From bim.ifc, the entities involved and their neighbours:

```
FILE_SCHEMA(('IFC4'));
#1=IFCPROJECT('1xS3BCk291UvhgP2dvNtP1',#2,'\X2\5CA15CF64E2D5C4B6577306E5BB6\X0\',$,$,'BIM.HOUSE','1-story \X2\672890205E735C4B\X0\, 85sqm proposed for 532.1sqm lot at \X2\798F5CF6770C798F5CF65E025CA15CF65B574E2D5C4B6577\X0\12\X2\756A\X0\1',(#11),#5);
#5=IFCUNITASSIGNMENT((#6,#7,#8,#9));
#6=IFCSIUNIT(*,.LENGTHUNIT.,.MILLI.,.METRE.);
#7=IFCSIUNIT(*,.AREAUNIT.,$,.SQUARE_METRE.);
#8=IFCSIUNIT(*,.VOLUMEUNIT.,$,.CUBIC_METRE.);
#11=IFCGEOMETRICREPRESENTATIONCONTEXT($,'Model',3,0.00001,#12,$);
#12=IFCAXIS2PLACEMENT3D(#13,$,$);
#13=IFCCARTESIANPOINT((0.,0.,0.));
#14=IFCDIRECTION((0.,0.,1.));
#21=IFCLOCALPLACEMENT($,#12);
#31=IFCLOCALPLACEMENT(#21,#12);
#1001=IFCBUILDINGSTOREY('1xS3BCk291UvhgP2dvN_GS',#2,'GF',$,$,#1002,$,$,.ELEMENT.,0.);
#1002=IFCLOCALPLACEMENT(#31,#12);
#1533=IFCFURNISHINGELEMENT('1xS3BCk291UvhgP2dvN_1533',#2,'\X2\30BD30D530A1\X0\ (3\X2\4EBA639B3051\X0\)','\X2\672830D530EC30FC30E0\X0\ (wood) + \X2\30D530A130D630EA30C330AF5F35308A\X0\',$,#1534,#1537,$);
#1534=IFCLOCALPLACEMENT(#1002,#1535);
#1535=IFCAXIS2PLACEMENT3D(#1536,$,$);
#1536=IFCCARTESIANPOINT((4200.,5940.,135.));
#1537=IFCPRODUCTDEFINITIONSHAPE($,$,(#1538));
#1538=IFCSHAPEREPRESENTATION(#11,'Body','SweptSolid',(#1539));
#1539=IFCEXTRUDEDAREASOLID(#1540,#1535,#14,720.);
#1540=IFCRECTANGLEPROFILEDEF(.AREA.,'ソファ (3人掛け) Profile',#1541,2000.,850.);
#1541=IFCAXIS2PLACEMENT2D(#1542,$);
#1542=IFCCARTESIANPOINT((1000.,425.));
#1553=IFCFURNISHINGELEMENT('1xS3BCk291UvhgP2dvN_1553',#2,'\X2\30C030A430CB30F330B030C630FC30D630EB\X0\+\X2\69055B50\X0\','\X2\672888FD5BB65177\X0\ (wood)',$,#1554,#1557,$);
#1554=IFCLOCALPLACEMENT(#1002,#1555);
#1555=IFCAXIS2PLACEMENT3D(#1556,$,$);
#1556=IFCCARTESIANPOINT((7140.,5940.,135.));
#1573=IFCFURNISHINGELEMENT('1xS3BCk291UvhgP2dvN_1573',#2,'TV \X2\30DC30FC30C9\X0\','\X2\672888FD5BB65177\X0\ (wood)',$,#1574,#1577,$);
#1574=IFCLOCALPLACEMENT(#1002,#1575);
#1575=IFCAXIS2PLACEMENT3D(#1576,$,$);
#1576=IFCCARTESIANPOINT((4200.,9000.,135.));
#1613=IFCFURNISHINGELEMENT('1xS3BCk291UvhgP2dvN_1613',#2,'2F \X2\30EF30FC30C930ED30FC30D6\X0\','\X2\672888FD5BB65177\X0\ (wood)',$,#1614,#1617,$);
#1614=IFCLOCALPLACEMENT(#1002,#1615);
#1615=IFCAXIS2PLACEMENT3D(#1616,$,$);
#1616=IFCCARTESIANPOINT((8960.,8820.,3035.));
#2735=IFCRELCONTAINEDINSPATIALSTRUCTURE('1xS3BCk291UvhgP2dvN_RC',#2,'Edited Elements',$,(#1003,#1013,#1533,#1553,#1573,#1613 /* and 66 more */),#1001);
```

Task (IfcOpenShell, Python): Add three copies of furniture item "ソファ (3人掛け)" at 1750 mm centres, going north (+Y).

```python
import numpy as np
import ifcopenshell
import ifcopenshell.api.geometry
import ifcopenshell.api.root
import ifcopenshell.util.element
import ifcopenshell.util.placement
import ifcopenshell.util.unit

model = ifcopenshell.open("bim.ifc")
unit_scale = ifcopenshell.util.unit.calculate_unit_scale(model)


def reuse_history(source, copy):
    """copy_class also copies each property set's owner history, people and application; keep the originals."""
    for rel in copy.IsDefinedBy:
        if rel.is_a("IfcRelDefinesByProperties") and (history := rel.RelatingPropertyDefinition.OwnerHistory):
            rel.RelatingPropertyDefinition.OwnerHistory = source.OwnerHistory
            ifcopenshell.util.element.remove_deep2(model, history)


source = model.by_guid("1xS3BCk291UvhgP2dvN_1533")
base = ifcopenshell.util.placement.get_local_placement(source.ObjectPlacement)
step = np.array([0.0, 1.0, 0.0]) * 1.75 / unit_scale

for i in range(1, 4):
    copy = ifcopenshell.api.root.copy_class(model, product=source)
    copy.Representation = ifcopenshell.util.element.copy_deep(
        model, source.Representation, exclude=["IfcGeometricRepresentationContext", "IfcRepresentationMap"]
    )
    reuse_history(source, copy)
    matrix = base.copy()
    matrix[:3, 3] += i * step
    print("added at", matrix[:3, 3].round(3) + 0.0)
    ifcopenshell.api.geometry.edit_object_placement(model, product=copy, matrix=matrix, is_si=False)

model.write("bim_edited.ifc")
```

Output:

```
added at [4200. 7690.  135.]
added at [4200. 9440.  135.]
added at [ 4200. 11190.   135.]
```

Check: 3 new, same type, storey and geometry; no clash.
